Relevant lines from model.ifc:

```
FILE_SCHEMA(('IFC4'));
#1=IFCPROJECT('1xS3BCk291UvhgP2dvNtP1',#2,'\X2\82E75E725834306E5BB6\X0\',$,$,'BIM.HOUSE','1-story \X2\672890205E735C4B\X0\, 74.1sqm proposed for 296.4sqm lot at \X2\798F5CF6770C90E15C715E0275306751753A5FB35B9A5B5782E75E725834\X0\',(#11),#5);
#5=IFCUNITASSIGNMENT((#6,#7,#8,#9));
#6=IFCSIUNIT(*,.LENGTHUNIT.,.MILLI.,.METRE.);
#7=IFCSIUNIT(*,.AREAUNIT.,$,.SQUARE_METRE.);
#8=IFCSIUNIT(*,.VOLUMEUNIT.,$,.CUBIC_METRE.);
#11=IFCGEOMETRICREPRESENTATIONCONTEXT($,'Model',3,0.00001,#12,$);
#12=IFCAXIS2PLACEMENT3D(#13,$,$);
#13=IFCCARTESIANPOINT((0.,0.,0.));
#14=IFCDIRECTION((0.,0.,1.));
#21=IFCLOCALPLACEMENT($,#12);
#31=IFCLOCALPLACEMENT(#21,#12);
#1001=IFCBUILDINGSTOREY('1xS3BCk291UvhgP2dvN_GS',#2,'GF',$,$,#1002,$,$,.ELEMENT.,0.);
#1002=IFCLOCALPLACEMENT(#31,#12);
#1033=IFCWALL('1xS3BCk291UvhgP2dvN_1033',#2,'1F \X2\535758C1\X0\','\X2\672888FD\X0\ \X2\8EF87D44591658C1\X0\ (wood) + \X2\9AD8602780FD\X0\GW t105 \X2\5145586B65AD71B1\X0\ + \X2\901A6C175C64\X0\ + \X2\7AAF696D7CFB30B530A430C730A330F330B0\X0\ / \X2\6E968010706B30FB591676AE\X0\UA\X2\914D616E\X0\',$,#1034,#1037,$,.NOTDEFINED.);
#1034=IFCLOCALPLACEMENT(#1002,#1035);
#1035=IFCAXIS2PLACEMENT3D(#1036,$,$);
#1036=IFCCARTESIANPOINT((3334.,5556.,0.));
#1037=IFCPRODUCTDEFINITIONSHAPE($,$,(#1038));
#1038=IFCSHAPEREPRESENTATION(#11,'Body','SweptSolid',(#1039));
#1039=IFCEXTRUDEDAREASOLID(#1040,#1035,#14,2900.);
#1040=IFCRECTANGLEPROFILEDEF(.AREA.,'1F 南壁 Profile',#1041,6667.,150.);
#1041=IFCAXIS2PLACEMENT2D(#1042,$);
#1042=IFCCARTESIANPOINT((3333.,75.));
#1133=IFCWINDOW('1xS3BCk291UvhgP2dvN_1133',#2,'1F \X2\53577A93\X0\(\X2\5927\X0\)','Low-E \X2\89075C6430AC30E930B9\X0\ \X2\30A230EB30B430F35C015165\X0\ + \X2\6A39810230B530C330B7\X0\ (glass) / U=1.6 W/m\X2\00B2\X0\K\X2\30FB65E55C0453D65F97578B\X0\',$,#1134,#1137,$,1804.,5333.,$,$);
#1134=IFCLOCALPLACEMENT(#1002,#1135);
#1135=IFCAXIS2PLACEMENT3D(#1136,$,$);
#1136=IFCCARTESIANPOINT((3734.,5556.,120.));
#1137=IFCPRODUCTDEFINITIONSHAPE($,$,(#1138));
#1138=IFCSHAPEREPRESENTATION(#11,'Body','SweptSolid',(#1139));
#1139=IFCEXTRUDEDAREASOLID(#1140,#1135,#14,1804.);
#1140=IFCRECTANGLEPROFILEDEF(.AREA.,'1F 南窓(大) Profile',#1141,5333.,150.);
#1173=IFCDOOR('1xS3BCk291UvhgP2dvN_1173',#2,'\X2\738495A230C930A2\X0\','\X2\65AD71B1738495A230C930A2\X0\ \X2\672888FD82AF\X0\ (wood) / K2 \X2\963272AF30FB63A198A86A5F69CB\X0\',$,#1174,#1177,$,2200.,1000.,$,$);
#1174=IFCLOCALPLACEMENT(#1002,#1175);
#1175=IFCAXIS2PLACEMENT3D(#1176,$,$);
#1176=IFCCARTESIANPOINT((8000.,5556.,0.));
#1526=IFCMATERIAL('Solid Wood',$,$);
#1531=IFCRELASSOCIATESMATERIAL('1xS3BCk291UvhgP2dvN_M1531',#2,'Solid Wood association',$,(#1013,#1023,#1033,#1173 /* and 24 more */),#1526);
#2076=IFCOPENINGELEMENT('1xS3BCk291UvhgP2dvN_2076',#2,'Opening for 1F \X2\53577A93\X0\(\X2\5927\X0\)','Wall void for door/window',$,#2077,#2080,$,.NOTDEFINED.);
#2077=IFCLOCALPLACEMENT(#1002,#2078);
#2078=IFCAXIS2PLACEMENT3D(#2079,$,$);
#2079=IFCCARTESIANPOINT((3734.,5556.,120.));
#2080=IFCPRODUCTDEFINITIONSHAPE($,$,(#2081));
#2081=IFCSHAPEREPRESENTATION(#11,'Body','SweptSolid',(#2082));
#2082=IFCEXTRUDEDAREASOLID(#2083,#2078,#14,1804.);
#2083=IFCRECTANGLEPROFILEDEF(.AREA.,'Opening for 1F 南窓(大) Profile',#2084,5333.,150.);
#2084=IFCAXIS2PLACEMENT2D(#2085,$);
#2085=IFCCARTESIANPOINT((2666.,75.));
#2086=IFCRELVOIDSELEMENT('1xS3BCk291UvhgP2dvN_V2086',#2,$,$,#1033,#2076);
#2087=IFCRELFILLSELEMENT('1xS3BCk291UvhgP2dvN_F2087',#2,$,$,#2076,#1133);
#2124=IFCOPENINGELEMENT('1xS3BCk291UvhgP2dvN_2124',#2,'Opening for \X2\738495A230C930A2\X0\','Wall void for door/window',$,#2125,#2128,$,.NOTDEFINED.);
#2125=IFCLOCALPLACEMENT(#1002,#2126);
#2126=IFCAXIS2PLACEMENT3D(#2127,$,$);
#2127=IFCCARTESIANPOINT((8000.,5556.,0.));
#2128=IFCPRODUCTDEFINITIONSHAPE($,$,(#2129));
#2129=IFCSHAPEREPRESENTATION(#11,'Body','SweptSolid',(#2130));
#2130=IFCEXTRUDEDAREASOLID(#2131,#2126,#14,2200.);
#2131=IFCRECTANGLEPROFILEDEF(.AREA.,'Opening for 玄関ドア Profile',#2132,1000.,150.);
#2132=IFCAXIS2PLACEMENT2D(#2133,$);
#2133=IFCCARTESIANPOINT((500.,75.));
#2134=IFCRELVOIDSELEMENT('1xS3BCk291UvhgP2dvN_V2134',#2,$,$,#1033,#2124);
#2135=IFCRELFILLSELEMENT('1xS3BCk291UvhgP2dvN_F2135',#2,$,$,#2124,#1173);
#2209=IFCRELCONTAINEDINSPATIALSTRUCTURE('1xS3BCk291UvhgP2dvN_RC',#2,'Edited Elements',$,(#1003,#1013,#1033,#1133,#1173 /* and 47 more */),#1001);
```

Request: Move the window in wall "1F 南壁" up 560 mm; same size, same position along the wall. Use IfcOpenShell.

```python
import numpy as np
import ifcopenshell
import ifcopenshell.api.geometry
import ifcopenshell.util.placement
import ifcopenshell.util.unit

model = ifcopenshell.open("model.ifc")
unit_scale = ifcopenshell.util.unit.calculate_unit_scale(model)

window = model.by_id(1133)
opening = window.FillsVoids[0].RelatingOpeningElement
dz = 0.56 / unit_scale

shift = np.array([0.0, 0.0, dz])
# The window is not placed relative to its opening, so move both.
for product in (opening, window):
    matrix = ifcopenshell.util.placement.get_local_placement(product.ObjectPlacement)
    matrix[:3, 3] += shift
    ifcopenshell.api.geometry.edit_object_placement(model, product=product, matrix=matrix, is_si=False)

print(f"moved by {dz * unit_scale:+.3f} m")

model.write("model_updated.ifc")
```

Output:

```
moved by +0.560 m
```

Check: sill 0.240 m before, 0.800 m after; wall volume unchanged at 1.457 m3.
